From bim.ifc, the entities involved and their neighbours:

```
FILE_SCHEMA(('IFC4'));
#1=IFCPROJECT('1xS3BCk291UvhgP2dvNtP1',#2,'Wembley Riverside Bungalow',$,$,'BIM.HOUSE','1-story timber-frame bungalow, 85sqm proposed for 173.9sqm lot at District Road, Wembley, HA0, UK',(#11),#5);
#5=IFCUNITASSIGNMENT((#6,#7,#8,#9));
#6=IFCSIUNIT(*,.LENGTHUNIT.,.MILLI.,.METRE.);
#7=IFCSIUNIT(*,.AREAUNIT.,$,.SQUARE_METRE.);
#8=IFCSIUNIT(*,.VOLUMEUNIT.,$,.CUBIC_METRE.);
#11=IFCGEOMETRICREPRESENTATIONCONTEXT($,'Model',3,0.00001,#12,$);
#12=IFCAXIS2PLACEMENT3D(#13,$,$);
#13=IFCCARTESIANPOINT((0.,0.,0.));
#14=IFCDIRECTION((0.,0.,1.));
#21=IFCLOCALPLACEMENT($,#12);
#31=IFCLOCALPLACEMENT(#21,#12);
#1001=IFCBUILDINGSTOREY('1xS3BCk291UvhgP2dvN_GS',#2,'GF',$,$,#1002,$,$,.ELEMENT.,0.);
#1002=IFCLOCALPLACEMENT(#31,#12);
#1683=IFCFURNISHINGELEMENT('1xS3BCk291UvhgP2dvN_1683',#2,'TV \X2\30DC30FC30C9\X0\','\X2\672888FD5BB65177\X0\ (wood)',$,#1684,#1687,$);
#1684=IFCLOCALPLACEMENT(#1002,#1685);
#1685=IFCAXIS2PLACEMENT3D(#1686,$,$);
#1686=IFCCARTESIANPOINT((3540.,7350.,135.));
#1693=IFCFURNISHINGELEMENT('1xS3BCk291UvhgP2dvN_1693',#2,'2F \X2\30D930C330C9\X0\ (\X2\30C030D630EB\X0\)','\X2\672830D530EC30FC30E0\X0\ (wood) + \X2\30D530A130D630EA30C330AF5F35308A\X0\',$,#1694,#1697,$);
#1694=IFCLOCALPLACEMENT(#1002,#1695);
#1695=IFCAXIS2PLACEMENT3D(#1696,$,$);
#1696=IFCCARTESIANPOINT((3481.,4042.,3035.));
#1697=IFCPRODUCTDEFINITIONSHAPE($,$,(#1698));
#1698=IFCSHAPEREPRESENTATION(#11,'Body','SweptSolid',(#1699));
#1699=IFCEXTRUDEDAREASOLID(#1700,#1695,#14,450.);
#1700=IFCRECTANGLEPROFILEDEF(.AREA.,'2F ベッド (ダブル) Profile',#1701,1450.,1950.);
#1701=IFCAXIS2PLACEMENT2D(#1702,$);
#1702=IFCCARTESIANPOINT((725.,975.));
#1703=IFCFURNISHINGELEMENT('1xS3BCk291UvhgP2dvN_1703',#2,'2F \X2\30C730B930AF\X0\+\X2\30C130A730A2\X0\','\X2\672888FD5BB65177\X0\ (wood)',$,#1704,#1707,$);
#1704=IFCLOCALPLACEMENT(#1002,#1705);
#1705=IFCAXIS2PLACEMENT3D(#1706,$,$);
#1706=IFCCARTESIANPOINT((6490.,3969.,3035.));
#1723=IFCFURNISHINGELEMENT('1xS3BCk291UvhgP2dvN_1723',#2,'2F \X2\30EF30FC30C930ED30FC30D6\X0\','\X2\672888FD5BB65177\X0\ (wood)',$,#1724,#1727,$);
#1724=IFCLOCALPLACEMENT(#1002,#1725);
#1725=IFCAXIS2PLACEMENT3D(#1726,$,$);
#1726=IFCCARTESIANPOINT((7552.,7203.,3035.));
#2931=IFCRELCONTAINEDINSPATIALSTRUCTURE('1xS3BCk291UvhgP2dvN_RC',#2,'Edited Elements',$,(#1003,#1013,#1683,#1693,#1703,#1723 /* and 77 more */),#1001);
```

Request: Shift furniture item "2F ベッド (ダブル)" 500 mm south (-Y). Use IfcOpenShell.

```python
import ifcopenshell
import ifcopenshell.api.geometry
import ifcopenshell.util.placement
import ifcopenshell.util.unit

model = ifcopenshell.open("bim.ifc")
unit_scale = ifcopenshell.util.unit.calculate_unit_scale(model)

item = model.by_guid("1xS3BCk291UvhgP2dvN_1693")
matrix = ifcopenshell.util.placement.get_local_placement(item.ObjectPlacement)
matrix[1, 3] -= 0.5 / unit_scale
ifcopenshell.api.geometry.edit_object_placement(model, product=item, matrix=matrix, is_si=False)

print(ifcopenshell.util.placement.get_local_placement(item.ObjectPlacement).round(3) + 0.0)

model.write("bim_rev.ifc")
```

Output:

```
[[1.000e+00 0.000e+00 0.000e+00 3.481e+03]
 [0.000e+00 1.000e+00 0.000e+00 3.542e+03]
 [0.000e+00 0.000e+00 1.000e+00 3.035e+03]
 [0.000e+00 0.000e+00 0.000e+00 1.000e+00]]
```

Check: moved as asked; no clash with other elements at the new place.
